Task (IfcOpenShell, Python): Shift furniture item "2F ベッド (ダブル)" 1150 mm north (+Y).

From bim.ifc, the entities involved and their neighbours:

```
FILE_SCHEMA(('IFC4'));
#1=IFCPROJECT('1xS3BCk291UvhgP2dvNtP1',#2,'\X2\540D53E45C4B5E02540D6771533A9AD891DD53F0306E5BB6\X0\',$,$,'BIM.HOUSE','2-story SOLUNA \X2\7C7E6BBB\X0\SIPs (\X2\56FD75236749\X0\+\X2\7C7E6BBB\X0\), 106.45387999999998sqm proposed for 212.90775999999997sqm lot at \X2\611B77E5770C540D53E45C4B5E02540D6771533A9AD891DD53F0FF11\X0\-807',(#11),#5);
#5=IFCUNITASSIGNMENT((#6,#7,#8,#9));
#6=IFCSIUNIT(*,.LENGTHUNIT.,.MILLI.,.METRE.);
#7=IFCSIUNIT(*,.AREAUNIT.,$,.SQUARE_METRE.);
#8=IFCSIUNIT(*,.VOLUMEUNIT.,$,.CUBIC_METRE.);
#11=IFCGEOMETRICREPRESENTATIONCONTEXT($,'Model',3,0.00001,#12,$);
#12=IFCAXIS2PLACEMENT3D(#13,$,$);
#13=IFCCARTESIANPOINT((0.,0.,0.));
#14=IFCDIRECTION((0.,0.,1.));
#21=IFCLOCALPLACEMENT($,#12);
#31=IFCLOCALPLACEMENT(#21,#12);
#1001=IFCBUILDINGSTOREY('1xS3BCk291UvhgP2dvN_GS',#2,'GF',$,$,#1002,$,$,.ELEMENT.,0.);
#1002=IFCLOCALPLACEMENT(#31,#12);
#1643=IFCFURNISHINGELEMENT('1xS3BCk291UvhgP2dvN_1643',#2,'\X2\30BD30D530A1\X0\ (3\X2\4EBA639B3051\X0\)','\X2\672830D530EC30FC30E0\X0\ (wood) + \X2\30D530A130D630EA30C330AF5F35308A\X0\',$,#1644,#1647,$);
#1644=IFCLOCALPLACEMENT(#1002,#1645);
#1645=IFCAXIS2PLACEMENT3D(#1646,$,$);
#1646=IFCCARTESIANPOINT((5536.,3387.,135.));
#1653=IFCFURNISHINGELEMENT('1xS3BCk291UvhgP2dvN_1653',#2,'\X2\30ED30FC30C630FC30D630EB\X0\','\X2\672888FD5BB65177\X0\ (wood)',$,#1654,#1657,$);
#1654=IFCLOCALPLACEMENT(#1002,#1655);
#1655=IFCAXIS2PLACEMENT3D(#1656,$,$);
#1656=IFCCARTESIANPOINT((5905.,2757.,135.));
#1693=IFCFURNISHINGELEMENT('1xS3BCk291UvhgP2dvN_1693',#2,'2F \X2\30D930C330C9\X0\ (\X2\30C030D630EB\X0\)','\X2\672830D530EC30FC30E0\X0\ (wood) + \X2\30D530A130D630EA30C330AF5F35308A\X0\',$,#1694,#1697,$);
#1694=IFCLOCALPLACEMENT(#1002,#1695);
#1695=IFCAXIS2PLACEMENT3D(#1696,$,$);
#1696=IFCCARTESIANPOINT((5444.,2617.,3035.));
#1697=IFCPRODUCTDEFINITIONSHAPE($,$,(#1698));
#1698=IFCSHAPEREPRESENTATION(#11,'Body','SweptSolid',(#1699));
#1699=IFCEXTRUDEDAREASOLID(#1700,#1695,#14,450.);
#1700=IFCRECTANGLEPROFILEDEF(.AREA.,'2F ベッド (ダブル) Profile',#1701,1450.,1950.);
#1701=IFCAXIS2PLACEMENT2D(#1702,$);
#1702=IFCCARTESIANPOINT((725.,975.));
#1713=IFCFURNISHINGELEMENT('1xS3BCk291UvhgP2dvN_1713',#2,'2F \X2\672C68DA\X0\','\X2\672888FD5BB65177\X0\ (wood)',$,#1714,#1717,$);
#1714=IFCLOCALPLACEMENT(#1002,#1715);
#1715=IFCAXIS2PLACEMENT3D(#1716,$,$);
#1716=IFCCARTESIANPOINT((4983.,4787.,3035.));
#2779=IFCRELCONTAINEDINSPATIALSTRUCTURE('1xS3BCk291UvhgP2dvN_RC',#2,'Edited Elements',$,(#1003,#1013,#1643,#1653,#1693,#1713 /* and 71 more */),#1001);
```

```python
import ifcopenshell
import ifcopenshell.api.geometry
import ifcopenshell.util.placement
import ifcopenshell.util.unit

model = ifcopenshell.open("bim.ifc")
unit_scale = ifcopenshell.util.unit.calculate_unit_scale(model)

item = model.by_guid("1xS3BCk291UvhgP2dvN_1693")
matrix = ifcopenshell.util.placement.get_local_placement(item.ObjectPlacement)
matrix[1, 3] += 1.15 / unit_scale
ifcopenshell.api.geometry.edit_object_placement(model, product=item, matrix=matrix, is_si=False)

print(ifcopenshell.util.placement.get_local_placement(item.ObjectPlacement).round(3) + 0.0)

model.write("bim_v2.ifc")
```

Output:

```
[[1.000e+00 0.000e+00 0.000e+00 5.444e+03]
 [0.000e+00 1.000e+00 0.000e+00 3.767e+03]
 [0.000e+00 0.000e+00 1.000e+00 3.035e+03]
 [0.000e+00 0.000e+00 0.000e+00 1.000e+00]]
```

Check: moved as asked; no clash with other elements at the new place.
